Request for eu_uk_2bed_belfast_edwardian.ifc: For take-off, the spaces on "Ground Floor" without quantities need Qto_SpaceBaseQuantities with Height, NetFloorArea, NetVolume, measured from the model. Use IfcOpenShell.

First a look at what the model holds.

```python
import ifcopenshell
import ifcopenshell.util.element
import ifcopenshell.util.unit

model = ifcopenshell.open("eu_uk_2bed_belfast_edwardian.ifc")
print(model.schema)
for unit_type in ("LENGTHUNIT", "AREAUNIT", "VOLUMEUNIT"):
    print(unit_type, ifcopenshell.util.unit.calculate_unit_scale(model, unit_type))
storey = next(s for s in model.by_type("IfcBuildingStorey") if s.Name == "Ground Floor")
spaces = [e for e in ifcopenshell.util.element.get_decomposition(storey) if e.is_a("IfcSpace")]
for e in sorted(spaces, key=lambda e: e.id()):
    print(e.id(), e.is_a(), e.Name, list(ifcopenshell.util.element.get_psets(e, qtos_only=True)), sep=" | ")
```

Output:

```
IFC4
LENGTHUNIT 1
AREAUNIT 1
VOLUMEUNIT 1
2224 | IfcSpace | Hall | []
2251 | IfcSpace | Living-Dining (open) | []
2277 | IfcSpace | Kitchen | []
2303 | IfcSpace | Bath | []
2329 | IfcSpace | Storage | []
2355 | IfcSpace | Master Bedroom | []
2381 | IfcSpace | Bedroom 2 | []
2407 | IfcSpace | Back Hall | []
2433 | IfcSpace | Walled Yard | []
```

```python
import ifcopenshell
import ifcopenshell.api.pset
import ifcopenshell.geom
import ifcopenshell.util.element
import ifcopenshell.util.shape
import ifcopenshell.util.unit

model = ifcopenshell.open("eu_uk_2bed_belfast_edwardian.ifc")
unit_scale = ifcopenshell.util.unit.calculate_unit_scale(model)
area_scale = ifcopenshell.util.unit.calculate_unit_scale(model, "AREAUNIT")
volume_scale = ifcopenshell.util.unit.calculate_unit_scale(model, "VOLUMEUNIT")
settings = ifcopenshell.geom.settings()

storey = next(s for s in model.by_type("IfcBuildingStorey") if s.Name == "Ground Floor")
spaces = [e for e in ifcopenshell.util.element.get_decomposition(storey) if e.is_a("IfcSpace")]

for e in sorted(spaces, key=lambda e: e.id()):
    if ifcopenshell.util.element.get_psets(e, qtos_only=True, should_inherit=False):
        continue
    # Geometry comes back in metres, in the element's own axes.
    shape = ifcopenshell.geom.create_shape(settings, e)
    values = {
        "Height": ifcopenshell.util.shape.get_z(shape.geometry) / unit_scale,
        "NetFloorArea": ifcopenshell.util.shape.get_footprint_area(shape.geometry) / area_scale,
        "NetVolume": ifcopenshell.util.shape.get_volume(shape.geometry) / volume_scale,
    }
    qto = ifcopenshell.api.pset.add_qto(model, product=e, name="Qto_SpaceBaseQuantities")
    ifcopenshell.api.pset.edit_qto(model, qto=qto, properties=values)
    print(e.id(), {k: round(v, 3) for k, v in values.items()})

model.write("eu_uk_2bed_belfast_edwardian_v2.ifc")
```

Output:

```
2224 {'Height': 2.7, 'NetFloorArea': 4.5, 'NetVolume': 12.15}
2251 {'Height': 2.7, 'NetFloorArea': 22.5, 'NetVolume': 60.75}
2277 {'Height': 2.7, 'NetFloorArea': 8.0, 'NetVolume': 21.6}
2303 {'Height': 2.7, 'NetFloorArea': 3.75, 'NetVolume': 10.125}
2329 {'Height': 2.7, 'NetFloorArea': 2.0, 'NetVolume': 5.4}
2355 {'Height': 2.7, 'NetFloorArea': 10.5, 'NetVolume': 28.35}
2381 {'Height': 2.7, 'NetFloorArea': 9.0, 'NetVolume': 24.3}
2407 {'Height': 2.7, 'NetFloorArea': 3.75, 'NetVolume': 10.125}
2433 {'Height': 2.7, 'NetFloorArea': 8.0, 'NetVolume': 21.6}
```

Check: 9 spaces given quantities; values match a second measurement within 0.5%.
